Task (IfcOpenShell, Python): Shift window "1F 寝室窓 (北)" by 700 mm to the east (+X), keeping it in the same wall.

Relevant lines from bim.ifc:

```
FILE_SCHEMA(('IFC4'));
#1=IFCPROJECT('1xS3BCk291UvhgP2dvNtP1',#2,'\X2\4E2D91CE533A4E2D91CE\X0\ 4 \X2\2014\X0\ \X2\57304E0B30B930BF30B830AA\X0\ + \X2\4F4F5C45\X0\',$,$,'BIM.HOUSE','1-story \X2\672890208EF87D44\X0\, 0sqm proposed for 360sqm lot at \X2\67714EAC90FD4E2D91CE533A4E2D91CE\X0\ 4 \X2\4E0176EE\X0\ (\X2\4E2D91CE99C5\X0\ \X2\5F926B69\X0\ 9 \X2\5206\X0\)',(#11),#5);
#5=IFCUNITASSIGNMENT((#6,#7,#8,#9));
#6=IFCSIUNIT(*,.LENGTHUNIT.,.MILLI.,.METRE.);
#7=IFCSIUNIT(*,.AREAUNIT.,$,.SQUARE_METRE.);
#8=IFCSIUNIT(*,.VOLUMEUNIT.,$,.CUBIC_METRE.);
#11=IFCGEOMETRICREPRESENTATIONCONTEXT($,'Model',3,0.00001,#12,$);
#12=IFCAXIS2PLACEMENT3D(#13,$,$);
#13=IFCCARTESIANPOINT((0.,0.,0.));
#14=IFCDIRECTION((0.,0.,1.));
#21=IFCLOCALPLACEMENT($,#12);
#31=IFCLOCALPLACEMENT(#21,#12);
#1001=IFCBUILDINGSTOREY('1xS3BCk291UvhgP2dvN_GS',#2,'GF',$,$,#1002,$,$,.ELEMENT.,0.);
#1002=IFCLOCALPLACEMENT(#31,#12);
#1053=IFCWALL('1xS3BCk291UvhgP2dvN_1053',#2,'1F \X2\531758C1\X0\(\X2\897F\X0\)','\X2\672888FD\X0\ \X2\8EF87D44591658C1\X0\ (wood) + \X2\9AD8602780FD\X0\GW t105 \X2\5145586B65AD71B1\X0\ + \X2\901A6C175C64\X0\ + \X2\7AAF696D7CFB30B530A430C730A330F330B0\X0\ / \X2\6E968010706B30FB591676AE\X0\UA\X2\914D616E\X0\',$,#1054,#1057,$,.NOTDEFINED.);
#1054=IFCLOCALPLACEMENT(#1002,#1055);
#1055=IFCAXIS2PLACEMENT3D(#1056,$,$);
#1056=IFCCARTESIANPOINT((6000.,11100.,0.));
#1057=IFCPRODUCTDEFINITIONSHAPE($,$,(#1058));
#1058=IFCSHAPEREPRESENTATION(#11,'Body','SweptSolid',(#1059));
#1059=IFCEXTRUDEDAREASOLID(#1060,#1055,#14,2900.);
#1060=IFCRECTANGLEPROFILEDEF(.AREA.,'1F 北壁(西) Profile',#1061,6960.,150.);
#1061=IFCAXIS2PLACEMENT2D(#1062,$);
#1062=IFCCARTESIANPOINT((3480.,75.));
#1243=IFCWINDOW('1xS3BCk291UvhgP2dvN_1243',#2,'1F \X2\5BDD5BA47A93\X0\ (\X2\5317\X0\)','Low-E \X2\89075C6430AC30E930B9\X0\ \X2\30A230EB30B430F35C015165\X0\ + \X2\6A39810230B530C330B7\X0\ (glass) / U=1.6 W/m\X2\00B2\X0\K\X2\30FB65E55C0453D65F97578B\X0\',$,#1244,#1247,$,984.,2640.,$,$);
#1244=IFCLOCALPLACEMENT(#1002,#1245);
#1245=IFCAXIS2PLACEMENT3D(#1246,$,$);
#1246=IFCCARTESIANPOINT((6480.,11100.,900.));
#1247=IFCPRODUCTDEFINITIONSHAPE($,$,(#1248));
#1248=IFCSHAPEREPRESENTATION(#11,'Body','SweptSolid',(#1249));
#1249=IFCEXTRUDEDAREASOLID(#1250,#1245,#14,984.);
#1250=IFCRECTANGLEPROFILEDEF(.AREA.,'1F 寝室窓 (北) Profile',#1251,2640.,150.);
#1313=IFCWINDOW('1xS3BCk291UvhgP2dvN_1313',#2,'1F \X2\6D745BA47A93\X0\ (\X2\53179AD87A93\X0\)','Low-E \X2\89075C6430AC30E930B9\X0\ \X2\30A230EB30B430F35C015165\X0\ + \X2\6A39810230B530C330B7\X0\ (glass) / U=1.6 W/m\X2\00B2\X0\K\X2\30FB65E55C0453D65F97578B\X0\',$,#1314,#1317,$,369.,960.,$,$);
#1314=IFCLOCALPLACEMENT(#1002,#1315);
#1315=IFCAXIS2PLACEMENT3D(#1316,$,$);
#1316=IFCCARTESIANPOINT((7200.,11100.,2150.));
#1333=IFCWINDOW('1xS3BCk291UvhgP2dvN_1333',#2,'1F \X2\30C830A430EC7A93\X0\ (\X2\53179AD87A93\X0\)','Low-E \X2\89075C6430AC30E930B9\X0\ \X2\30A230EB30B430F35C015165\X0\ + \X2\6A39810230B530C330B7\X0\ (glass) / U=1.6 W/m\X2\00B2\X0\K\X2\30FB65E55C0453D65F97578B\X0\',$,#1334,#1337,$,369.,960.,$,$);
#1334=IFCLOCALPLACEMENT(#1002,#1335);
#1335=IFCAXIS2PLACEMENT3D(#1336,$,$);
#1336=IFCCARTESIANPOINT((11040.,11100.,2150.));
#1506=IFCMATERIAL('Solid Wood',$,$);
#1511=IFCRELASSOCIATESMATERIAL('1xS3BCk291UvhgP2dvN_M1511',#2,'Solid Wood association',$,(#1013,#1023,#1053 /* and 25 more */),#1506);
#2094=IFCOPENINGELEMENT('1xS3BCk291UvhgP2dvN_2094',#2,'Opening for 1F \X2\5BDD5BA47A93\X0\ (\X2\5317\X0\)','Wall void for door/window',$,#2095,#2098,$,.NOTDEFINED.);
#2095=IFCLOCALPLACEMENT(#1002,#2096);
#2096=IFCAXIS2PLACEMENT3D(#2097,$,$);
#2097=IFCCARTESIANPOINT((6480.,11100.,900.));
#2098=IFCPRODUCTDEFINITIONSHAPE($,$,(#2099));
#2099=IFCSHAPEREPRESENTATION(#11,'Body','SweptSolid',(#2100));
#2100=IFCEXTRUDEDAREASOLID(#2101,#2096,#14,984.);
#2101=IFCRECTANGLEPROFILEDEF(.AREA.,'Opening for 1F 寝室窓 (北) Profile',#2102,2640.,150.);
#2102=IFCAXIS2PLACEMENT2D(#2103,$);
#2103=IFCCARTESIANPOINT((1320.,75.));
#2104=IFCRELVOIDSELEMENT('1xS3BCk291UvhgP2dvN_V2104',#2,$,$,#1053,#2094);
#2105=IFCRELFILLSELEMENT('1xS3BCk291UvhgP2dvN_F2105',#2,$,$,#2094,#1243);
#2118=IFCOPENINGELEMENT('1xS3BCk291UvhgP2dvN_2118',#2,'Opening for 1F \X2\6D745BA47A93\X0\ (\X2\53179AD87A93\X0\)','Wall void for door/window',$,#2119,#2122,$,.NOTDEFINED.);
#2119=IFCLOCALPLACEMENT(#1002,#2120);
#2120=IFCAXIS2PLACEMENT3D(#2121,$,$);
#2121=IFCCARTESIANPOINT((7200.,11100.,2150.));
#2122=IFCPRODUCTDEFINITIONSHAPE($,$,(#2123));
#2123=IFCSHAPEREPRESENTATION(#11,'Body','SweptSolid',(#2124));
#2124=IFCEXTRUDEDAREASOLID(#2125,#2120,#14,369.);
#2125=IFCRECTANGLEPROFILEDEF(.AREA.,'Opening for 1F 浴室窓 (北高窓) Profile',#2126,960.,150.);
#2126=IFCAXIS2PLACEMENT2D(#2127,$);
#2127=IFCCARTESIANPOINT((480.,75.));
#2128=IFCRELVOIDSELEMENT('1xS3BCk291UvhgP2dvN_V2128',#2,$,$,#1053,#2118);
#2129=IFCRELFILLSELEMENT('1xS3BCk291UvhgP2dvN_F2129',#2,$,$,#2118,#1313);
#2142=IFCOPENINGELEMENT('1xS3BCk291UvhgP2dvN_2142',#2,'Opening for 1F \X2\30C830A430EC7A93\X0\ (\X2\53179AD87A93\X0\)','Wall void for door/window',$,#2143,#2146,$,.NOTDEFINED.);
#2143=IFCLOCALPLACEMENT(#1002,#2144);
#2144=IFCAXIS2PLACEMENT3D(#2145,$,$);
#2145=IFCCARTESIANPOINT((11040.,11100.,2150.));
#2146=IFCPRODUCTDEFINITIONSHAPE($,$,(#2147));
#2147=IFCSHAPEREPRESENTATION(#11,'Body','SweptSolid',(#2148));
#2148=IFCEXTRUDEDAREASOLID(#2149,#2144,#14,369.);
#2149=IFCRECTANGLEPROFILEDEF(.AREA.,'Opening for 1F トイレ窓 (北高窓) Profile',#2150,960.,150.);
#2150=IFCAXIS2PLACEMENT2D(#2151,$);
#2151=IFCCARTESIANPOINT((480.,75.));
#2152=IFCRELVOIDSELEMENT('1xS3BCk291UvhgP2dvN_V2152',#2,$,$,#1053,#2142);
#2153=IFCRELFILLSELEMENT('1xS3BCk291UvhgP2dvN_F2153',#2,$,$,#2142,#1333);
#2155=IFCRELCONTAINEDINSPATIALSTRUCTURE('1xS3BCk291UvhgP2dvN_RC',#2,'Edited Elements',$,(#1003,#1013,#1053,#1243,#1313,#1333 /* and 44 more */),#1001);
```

```python
import ifcopenshell
import ifcopenshell.api.geometry
import ifcopenshell.util.placement

model = ifcopenshell.open("bim.ifc")

window = model.by_id(1243)
opening = window.FillsVoids[0].RelatingOpeningElement
wall = opening.VoidsElements[0].RelatingBuildingElement

wall_matrix = ifcopenshell.util.placement.get_local_placement(wall.ObjectPlacement)
shift = wall_matrix[:3, 0] * 700.0
before = ifcopenshell.util.placement.get_local_placement(window.ObjectPlacement)[:3, 3].copy()

# The window is not placed relative to its opening, so move both.
for product in (opening, window):
    matrix = ifcopenshell.util.placement.get_local_placement(product.ObjectPlacement)
    matrix[:3, 3] += shift
    ifcopenshell.api.geometry.edit_object_placement(model, product=product, matrix=matrix, is_si=False)

after = ifcopenshell.util.placement.get_local_placement(window.ObjectPlacement)[:3, 3]
print("window moved by", (after - before).round(3) + 0.0)

model.write("bim-out.ifc")
```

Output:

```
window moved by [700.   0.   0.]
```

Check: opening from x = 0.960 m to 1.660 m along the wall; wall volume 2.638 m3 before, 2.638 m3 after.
